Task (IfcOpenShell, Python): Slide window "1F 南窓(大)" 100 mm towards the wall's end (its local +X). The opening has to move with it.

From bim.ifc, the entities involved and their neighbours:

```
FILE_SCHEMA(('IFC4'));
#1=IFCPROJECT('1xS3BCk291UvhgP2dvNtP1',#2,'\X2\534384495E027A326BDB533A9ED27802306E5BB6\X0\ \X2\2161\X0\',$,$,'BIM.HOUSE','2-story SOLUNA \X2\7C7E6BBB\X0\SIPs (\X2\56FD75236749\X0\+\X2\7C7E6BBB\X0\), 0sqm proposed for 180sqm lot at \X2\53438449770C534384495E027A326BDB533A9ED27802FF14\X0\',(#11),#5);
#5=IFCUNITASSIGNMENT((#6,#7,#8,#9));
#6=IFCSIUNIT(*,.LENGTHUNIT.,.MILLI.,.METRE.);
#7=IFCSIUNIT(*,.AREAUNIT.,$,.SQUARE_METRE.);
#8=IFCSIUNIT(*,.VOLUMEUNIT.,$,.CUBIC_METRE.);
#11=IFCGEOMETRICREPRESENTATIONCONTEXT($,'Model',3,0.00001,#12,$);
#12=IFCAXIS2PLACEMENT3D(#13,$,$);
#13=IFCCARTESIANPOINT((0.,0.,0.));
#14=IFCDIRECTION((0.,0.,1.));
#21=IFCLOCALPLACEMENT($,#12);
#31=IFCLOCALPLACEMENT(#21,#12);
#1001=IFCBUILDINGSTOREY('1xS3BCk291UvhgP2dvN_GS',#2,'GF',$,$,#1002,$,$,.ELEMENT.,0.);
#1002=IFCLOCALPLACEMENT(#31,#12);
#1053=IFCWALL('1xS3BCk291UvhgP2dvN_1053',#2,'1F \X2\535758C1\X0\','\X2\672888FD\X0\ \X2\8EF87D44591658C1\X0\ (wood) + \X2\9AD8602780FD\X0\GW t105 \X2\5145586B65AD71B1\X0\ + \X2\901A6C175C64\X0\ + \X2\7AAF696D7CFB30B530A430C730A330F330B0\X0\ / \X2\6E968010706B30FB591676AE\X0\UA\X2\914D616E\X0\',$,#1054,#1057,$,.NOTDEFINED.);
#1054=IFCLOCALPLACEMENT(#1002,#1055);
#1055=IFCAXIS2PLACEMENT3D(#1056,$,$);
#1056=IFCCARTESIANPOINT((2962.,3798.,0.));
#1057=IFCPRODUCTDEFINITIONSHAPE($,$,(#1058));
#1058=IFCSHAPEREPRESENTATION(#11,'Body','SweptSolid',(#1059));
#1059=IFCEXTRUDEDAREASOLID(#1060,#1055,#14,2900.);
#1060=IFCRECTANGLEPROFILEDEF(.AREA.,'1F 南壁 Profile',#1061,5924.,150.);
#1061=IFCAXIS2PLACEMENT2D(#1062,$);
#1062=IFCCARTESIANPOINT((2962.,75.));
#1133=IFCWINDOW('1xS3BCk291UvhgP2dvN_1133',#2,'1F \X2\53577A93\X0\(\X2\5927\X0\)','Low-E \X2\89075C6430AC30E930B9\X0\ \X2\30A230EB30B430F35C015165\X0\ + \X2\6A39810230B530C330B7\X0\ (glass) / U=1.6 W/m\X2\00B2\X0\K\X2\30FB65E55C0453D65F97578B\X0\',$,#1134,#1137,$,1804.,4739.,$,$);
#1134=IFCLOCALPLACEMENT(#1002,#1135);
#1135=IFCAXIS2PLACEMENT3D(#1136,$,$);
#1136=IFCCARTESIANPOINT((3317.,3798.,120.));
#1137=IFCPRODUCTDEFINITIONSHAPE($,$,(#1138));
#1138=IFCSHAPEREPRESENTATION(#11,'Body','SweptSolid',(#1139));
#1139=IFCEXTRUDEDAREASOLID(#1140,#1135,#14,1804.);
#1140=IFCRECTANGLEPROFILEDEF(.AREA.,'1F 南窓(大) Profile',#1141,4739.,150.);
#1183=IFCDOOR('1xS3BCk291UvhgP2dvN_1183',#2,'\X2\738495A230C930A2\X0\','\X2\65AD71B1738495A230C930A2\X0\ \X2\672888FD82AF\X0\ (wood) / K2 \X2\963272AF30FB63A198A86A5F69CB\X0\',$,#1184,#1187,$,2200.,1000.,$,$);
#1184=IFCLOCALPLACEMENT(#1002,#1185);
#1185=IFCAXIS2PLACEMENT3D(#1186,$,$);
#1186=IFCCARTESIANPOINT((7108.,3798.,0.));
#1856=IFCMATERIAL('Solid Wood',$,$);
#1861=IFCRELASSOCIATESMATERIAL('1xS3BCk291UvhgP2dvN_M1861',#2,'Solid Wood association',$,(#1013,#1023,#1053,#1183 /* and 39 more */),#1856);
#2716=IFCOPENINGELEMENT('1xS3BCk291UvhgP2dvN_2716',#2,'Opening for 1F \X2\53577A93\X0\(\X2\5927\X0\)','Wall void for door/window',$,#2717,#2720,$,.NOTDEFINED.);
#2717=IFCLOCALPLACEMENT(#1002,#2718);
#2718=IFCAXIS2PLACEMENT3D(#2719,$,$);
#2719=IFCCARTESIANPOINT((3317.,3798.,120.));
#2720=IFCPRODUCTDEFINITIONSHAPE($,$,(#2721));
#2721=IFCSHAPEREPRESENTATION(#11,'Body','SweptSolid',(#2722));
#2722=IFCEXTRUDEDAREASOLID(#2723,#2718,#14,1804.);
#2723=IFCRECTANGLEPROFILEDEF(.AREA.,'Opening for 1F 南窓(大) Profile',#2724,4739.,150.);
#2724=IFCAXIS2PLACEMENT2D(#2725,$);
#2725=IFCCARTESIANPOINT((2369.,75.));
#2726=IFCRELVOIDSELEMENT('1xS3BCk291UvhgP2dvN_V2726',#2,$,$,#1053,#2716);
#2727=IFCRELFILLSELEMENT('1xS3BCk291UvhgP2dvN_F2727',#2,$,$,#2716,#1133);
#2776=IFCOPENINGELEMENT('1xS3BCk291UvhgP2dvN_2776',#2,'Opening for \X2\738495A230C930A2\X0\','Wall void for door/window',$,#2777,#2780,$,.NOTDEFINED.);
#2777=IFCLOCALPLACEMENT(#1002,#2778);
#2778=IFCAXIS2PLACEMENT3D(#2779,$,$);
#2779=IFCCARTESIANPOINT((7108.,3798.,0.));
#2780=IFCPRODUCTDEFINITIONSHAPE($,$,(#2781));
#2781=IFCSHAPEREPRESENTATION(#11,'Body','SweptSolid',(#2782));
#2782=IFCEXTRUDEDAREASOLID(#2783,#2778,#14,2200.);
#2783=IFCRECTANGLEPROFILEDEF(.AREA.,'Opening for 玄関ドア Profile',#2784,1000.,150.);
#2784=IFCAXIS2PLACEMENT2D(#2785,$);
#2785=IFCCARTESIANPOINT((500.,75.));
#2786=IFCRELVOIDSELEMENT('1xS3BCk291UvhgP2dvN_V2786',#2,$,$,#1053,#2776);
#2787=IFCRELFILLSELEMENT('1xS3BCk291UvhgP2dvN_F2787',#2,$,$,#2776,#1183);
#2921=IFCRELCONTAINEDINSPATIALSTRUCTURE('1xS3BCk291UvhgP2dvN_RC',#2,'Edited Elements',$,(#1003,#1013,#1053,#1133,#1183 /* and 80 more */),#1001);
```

```python
import ifcopenshell
import ifcopenshell.api.geometry
import ifcopenshell.util.placement

model = ifcopenshell.open("bim.ifc")

window = model.by_guid("1xS3BCk291UvhgP2dvN_1133")
opening = window.FillsVoids[0].RelatingOpeningElement
wall = opening.VoidsElements[0].RelatingBuildingElement

wall_matrix = ifcopenshell.util.placement.get_local_placement(wall.ObjectPlacement)
shift = wall_matrix[:3, 0] * 100.0
before = ifcopenshell.util.placement.get_local_placement(window.ObjectPlacement)[:3, 3].copy()

# The window is not placed relative to its opening, so move both.
for product in (opening, window):
    matrix = ifcopenshell.util.placement.get_local_placement(product.ObjectPlacement)
    matrix[:3, 3] += shift
    ifcopenshell.api.geometry.edit_object_placement(model, product=product, matrix=matrix, is_si=False)

after = ifcopenshell.util.placement.get_local_placement(window.ObjectPlacement)[:3, 3]
print("window moved by", (after - before).round(3) + 0.0)

model.write("bim_updated.ifc")
```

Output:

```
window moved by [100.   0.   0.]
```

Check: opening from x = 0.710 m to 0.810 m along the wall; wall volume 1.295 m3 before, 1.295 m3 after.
